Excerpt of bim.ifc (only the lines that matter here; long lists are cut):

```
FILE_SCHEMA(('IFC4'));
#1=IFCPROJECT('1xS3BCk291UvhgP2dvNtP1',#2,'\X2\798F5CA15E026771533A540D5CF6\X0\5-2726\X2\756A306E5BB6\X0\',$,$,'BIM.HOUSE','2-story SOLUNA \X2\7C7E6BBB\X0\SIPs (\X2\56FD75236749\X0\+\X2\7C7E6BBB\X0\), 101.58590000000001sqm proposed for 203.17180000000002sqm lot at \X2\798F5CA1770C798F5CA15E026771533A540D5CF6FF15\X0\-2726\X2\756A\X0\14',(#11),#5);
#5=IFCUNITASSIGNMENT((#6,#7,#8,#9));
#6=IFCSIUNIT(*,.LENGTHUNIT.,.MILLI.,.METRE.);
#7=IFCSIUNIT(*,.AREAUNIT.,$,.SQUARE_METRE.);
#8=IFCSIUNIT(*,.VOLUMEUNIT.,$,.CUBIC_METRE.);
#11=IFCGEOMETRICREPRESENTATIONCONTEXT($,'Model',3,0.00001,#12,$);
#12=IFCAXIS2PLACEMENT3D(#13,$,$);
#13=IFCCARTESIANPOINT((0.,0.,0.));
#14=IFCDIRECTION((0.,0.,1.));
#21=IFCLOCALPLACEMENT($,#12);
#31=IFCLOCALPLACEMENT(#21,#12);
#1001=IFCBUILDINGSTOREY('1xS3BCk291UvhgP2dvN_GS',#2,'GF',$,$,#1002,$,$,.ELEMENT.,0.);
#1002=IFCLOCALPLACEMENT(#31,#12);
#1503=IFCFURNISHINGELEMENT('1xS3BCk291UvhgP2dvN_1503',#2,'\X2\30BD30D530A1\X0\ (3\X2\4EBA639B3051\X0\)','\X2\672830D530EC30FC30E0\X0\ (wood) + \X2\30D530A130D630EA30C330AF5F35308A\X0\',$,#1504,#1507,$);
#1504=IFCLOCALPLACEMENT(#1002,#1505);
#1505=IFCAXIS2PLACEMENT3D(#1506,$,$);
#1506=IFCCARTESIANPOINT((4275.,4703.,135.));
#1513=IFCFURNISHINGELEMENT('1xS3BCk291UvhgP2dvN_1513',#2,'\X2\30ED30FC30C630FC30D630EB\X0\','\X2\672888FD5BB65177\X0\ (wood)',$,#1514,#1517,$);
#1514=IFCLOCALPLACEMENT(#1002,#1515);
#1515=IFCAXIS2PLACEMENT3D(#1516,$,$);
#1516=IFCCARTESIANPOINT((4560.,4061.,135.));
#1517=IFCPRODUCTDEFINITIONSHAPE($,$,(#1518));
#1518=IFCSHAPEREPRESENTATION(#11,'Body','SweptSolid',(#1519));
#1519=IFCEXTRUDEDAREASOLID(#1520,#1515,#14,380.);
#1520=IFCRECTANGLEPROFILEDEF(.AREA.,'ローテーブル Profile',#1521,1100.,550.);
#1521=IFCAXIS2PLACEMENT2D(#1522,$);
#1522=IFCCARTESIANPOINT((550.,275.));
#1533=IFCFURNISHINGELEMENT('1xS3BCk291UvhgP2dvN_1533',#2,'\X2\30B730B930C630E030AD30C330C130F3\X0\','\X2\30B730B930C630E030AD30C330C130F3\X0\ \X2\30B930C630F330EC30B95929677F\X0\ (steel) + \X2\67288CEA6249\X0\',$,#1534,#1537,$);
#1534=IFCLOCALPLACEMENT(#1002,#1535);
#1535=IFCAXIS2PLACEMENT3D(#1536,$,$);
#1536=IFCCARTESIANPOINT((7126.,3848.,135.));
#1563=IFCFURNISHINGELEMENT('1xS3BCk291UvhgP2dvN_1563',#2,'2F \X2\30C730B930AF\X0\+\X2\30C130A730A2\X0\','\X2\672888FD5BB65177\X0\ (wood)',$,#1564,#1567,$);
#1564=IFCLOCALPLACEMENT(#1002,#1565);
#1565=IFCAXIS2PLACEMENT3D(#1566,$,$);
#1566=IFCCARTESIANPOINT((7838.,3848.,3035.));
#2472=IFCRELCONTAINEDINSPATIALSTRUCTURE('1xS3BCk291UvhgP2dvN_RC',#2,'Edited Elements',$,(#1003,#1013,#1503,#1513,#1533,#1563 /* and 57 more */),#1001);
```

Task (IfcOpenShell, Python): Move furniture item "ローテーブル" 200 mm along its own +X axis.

```python
import ifcopenshell
import ifcopenshell.api.geometry
import ifcopenshell.util.placement
import ifcopenshell.util.unit

model = ifcopenshell.open("bim.ifc")
unit_scale = ifcopenshell.util.unit.calculate_unit_scale(model)

item = model.by_guid("1xS3BCk291UvhgP2dvN_1513")
matrix = ifcopenshell.util.placement.get_local_placement(item.ObjectPlacement)
matrix[:3, 3] += matrix[:3, 0] * 0.2 / unit_scale
ifcopenshell.api.geometry.edit_object_placement(model, product=item, matrix=matrix, is_si=False)

print(ifcopenshell.util.placement.get_local_placement(item.ObjectPlacement).round(3) + 0.0)

model.write("bim-out.ifc")
```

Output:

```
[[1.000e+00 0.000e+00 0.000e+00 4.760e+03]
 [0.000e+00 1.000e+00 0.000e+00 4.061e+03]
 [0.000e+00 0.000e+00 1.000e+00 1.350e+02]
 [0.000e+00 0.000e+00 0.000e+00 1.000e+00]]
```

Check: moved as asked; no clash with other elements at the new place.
